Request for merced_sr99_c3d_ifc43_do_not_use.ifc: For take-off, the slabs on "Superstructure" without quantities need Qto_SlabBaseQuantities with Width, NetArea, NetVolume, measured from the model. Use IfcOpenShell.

First a look at what the model holds.

```python
import ifcopenshell
import ifcopenshell.util.element
import ifcopenshell.util.unit

model = ifcopenshell.open("merced_sr99_c3d_ifc43_do_not_use.ifc")
print(model.schema)
for unit_type in ("LENGTHUNIT", "AREAUNIT", "VOLUMEUNIT"):
    print(unit_type, ifcopenshell.util.unit.calculate_unit_scale(model, unit_type))
storey = next(s for s in model.by_type("IfcBuildingStorey") if s.Name == "Superstructure")
slabs = [e for e in ifcopenshell.util.element.get_decomposition(storey) if e.is_a("IfcSlab")]
for e in sorted(slabs, key=lambda e: e.id()):
    print(e.id(), e.is_a(), e.Name, list(ifcopenshell.util.element.get_psets(e, qtos_only=True)), sep=" | ")
```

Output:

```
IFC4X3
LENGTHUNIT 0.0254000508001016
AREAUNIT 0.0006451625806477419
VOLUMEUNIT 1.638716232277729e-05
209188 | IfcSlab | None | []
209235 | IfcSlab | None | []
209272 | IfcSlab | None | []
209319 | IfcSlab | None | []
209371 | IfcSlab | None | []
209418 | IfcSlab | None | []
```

```python
import ifcopenshell
import ifcopenshell.api.pset
import ifcopenshell.geom
import ifcopenshell.util.element
import ifcopenshell.util.shape
import ifcopenshell.util.unit

model = ifcopenshell.open("merced_sr99_c3d_ifc43_do_not_use.ifc")
unit_scale = ifcopenshell.util.unit.calculate_unit_scale(model)
area_scale = ifcopenshell.util.unit.calculate_unit_scale(model, "AREAUNIT")
volume_scale = ifcopenshell.util.unit.calculate_unit_scale(model, "VOLUMEUNIT")
settings = ifcopenshell.geom.settings()

storey = next(s for s in model.by_type("IfcBuildingStorey") if s.Name == "Superstructure")
slabs = [e for e in ifcopenshell.util.element.get_decomposition(storey) if e.is_a("IfcSlab")]

for e in sorted(slabs, key=lambda e: e.id()):
    if ifcopenshell.util.element.get_psets(e, qtos_only=True, should_inherit=False):
        continue
    # Geometry comes back in metres, in the element's own axes.
    shape = ifcopenshell.geom.create_shape(settings, e)
    values = {
        "Width": ifcopenshell.util.shape.get_z(shape.geometry) / unit_scale,
        "NetArea": ifcopenshell.util.shape.get_footprint_area(shape.geometry) / area_scale,
        "NetVolume": ifcopenshell.util.shape.get_volume(shape.geometry) / volume_scale,
    }
    qto = ifcopenshell.api.pset.add_qto(model, product=e, name="Qto_SlabBaseQuantities")
    ifcopenshell.api.pset.edit_qto(model, qto=qto, properties=values)
    print(e.id(), {k: round(v, 3) for k, v in values.items()})

model.write("merced_sr99_c3d_ifc43_do_not_use_rev.ifc")
```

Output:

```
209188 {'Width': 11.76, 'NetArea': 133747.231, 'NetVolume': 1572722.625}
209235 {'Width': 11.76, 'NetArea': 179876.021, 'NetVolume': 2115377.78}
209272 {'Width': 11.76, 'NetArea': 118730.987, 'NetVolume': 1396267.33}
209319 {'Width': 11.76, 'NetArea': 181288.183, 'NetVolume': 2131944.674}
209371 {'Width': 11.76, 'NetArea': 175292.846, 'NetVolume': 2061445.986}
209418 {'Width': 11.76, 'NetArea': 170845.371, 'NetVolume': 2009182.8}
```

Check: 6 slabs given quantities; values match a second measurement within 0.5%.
